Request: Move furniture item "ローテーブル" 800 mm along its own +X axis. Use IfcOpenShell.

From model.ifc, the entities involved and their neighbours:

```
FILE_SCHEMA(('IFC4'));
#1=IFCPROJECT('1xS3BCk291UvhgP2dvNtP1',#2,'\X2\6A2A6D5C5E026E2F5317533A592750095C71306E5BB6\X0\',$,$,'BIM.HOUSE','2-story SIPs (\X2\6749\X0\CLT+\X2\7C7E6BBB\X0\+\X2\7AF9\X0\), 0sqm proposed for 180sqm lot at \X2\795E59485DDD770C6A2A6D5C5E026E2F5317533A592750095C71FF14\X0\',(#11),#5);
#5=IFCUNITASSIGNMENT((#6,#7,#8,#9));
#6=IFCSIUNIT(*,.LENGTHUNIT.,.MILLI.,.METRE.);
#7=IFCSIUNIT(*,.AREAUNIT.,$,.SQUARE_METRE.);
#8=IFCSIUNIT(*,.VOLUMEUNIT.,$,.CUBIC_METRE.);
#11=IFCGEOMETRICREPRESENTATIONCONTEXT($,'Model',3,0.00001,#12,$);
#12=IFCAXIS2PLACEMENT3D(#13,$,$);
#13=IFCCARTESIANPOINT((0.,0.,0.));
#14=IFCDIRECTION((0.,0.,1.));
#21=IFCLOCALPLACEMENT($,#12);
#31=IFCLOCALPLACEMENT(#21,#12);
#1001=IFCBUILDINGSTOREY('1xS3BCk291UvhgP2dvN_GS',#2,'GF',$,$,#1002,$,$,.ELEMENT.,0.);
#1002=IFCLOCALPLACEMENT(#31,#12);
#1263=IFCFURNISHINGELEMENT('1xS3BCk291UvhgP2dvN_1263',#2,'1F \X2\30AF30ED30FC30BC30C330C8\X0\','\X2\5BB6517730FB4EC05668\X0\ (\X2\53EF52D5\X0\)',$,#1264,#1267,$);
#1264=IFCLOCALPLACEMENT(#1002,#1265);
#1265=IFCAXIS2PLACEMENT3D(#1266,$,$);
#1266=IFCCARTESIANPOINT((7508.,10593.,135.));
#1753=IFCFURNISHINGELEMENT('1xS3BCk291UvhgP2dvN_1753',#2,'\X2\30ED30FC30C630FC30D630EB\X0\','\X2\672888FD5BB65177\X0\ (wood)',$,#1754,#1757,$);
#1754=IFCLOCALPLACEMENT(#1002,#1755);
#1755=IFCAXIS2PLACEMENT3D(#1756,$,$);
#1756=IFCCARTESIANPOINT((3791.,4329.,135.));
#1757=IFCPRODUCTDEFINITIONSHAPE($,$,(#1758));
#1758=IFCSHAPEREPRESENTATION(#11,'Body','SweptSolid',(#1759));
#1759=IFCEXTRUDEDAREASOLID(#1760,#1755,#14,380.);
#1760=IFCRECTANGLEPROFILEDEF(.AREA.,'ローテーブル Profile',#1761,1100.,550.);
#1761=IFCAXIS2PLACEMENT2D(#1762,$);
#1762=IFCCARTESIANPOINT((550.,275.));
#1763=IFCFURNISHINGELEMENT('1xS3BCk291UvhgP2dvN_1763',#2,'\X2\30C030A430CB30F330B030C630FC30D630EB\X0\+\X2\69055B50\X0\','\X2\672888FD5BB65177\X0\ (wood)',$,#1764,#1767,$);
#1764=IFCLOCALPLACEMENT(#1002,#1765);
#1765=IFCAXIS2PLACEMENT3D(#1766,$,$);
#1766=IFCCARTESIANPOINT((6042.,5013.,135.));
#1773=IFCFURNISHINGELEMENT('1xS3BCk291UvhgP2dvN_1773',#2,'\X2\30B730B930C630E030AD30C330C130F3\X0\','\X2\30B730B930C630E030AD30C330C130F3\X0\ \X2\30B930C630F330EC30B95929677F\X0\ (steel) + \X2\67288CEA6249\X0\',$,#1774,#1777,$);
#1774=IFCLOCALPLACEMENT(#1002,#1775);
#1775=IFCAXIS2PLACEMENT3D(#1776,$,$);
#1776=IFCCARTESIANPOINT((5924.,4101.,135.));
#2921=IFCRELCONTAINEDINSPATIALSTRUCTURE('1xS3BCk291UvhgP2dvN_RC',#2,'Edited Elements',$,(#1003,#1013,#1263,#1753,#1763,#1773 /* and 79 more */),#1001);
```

```python
import ifcopenshell
import ifcopenshell.api.geometry
import ifcopenshell.util.placement
import ifcopenshell.util.unit

model = ifcopenshell.open("model.ifc")
unit_scale = ifcopenshell.util.unit.calculate_unit_scale(model)

item = model.by_guid("1xS3BCk291UvhgP2dvN_1753")
matrix = ifcopenshell.util.placement.get_local_placement(item.ObjectPlacement)
matrix[:3, 3] += matrix[:3, 0] * 0.8 / unit_scale
ifcopenshell.api.geometry.edit_object_placement(model, product=item, matrix=matrix, is_si=False)

print(ifcopenshell.util.placement.get_local_placement(item.ObjectPlacement).round(3) + 0.0)

model.write("model_v2.ifc")
```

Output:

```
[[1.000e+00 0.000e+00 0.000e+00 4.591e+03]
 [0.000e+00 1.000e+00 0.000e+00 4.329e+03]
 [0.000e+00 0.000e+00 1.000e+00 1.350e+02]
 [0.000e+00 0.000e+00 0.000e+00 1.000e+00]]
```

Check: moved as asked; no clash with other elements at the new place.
